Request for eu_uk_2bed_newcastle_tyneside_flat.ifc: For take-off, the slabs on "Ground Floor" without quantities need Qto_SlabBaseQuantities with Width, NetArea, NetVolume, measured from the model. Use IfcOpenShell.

First a look at what the model holds.

```python
import ifcopenshell
import ifcopenshell.util.element
import ifcopenshell.util.unit

model = ifcopenshell.open("eu_uk_2bed_newcastle_tyneside_flat.ifc")
print(model.schema)
for unit_type in ("LENGTHUNIT", "AREAUNIT", "VOLUMEUNIT"):
    print(unit_type, ifcopenshell.util.unit.calculate_unit_scale(model, unit_type))
storey = next(s for s in model.by_type("IfcBuildingStorey") if s.Name == "Ground Floor")
slabs = [e for e in ifcopenshell.util.element.get_decomposition(storey) if e.is_a("IfcSlab")]
for e in sorted(slabs, key=lambda e: e.id()):
    print(e.id(), e.is_a(), e.Name, list(ifcopenshell.util.element.get_psets(e, qtos_only=True)), sep=" | ")
```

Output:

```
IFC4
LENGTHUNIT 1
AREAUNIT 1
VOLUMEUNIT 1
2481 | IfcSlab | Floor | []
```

```python
import ifcopenshell
import ifcopenshell.api.pset
import ifcopenshell.geom
import ifcopenshell.util.element
import ifcopenshell.util.shape
import ifcopenshell.util.unit

model = ifcopenshell.open("eu_uk_2bed_newcastle_tyneside_flat.ifc")
unit_scale = ifcopenshell.util.unit.calculate_unit_scale(model)
area_scale = ifcopenshell.util.unit.calculate_unit_scale(model, "AREAUNIT")
volume_scale = ifcopenshell.util.unit.calculate_unit_scale(model, "VOLUMEUNIT")
settings = ifcopenshell.geom.settings()

storey = next(s for s in model.by_type("IfcBuildingStorey") if s.Name == "Ground Floor")
slabs = [e for e in ifcopenshell.util.element.get_decomposition(storey) if e.is_a("IfcSlab")]

for e in sorted(slabs, key=lambda e: e.id()):
    if ifcopenshell.util.element.get_psets(e, qtos_only=True, should_inherit=False):
        continue
    # Geometry comes back in metres, in the element's own axes.
    shape = ifcopenshell.geom.create_shape(settings, e)
    values = {
        "Width": ifcopenshell.util.shape.get_z(shape.geometry) / unit_scale,
        "NetArea": ifcopenshell.util.shape.get_footprint_area(shape.geometry) / area_scale,
        "NetVolume": ifcopenshell.util.shape.get_volume(shape.geometry) / volume_scale,
    }
    qto = ifcopenshell.api.pset.add_qto(model, product=e, name="Qto_SlabBaseQuantities")
    ifcopenshell.api.pset.edit_qto(model, qto=qto, properties=values)
    print(e.id(), {k: round(v, 3) for k, v in values.items()})

model.write("eu_uk_2bed_newcastle_tyneside_flat-out.ifc")
```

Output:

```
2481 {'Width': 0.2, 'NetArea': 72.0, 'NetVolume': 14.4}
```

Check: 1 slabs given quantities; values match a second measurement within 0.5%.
